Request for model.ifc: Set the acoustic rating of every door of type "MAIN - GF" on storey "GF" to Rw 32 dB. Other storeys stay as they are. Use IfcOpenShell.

First a look at what the model holds.

```python
import ifcopenshell
import ifcopenshell.util.element

model = ifcopenshell.open("model.ifc")
print(model.schema)
storey = next(s for s in model.by_type("IfcBuildingStorey") if s.Name == "GF")
doors = [e for e in ifcopenshell.util.element.get_decomposition(storey) if e.is_a("IfcDoor")]
seen = {}
for e in doors:
    element_type = ifcopenshell.util.element.get_type(e)
    key = (element_type.Name if element_type != e and element_type else None, ifcopenshell.util.element.get_pset(e, "Pset_DoorCommon", "AcousticRating"))
    seen[key] = seen.get(key, 0) + 1
for (name, value), count in sorted(seen.items(), key=str):
    print(count, "x", name, "|", value)
```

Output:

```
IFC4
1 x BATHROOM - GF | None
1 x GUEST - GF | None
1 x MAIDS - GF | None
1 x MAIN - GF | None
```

```python
import ifcopenshell
import ifcopenshell.api.pset
import ifcopenshell.util.element

model = ifcopenshell.open("model.ifc")

storey = next(s for s in model.by_type("IfcBuildingStorey") if s.Name == "GF")
doors = [e for e in ifcopenshell.util.element.get_decomposition(storey) if e.is_a("IfcDoor")]

count = 0
for e in doors:
    element_type = ifcopenshell.util.element.get_type(e)
    if element_type in (None, e) or element_type.Name != "MAIN - GF":
        continue
    # add_pset returns the element's existing set when there is one.
    pset = ifcopenshell.api.pset.add_pset(model, product=e, name="Pset_DoorCommon")
    ifcopenshell.api.pset.edit_pset(model, pset=pset, properties={"AcousticRating": "Rw 32 dB"})
    count += 1

print(count, "doors updated")

model.write("model_updated.ifc")
```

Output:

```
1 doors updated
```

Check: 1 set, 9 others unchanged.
